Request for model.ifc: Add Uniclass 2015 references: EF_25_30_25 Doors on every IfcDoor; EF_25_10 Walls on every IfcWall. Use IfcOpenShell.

First a look at what the model holds.

```python
import ifcopenshell

model = ifcopenshell.open("model.ifc")
print(model.schema)
print("classifications:", [c.Name for c in model.by_type("IfcClassification")])
for ifc_class in ("IfcDoor", "IfcRoof", "IfcStair", "IfcWall", "IfcWindow"):
    print(ifc_class, len(model.by_type(ifc_class)))
```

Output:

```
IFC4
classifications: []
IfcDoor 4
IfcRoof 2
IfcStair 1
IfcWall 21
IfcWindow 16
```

```python
import ifcopenshell
import ifcopenshell.api.classification

model = ifcopenshell.open("model.ifc")

system = ifcopenshell.api.classification.add_classification(model, classification="Uniclass 2015")

codes = {
    "IfcDoor": ("EF_25_30_25", "Doors"),
    "IfcWall": ("EF_25_10", "Walls"),
}
for ifc_class, (code, name) in codes.items():
    products = model.by_type(ifc_class)
    ifcopenshell.api.classification.add_reference(
        model, products=products, classification=system, identification=code, name=name
    )
    print(code, len(products))

model.write("model_edited.ifc")
```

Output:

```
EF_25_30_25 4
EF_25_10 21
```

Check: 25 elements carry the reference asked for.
